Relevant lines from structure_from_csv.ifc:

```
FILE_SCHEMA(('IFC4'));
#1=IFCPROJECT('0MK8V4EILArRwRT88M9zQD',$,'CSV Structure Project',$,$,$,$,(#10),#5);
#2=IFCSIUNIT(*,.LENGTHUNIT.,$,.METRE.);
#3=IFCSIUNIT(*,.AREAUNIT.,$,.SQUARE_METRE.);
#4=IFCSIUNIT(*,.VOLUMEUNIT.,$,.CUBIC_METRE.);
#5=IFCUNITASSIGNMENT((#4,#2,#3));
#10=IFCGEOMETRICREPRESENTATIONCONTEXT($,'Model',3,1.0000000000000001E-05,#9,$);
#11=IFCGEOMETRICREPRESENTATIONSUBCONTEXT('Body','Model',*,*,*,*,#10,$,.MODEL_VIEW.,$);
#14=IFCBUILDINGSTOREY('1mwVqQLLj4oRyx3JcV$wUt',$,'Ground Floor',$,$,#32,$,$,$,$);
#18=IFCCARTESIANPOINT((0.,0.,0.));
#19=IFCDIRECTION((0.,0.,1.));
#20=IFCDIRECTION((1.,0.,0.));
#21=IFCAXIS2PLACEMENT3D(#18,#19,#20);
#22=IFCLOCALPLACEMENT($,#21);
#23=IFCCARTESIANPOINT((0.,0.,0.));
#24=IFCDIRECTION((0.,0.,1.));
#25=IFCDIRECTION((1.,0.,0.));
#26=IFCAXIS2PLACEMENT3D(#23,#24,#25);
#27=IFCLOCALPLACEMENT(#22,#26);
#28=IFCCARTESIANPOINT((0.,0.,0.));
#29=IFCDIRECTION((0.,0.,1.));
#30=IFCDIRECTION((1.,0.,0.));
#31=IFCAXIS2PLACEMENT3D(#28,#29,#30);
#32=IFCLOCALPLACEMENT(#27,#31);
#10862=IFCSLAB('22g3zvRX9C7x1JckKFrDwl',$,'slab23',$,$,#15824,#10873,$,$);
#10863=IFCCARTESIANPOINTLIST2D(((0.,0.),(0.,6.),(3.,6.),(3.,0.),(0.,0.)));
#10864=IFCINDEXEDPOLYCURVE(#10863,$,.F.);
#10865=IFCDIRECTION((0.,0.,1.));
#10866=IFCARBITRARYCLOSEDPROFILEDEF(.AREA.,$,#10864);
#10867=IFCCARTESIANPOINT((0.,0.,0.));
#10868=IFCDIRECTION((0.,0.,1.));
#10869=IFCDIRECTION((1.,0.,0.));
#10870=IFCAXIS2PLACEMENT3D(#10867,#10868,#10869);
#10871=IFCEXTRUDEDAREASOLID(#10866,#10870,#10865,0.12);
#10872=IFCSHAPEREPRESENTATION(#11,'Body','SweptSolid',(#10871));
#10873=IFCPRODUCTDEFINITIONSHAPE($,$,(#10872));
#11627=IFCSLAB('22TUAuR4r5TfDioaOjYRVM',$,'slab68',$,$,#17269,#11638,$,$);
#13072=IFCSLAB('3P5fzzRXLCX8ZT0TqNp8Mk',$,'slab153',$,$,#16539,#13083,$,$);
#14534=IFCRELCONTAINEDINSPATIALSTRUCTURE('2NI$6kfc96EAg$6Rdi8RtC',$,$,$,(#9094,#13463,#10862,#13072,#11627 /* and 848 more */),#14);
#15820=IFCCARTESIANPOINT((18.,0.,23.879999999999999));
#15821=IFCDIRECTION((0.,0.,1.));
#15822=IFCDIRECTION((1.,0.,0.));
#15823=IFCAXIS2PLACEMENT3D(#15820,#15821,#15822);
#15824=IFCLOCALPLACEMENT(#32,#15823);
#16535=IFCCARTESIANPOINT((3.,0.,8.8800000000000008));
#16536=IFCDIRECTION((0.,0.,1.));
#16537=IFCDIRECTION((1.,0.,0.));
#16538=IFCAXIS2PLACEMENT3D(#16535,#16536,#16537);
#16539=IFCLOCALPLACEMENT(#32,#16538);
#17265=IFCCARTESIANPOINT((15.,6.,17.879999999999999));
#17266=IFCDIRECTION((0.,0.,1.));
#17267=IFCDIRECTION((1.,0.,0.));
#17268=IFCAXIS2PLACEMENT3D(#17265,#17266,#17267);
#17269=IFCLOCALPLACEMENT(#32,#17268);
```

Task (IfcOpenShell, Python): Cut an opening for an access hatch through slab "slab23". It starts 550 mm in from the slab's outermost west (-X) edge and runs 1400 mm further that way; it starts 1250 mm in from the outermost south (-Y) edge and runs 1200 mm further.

```python
import numpy as np
import ifcopenshell
import ifcopenshell.api.feature
import ifcopenshell.api.geometry
import ifcopenshell.api.root
import ifcopenshell.geom
import ifcopenshell.util.placement
import ifcopenshell.util.representation
import ifcopenshell.util.shape
import ifcopenshell.util.unit

model = ifcopenshell.open("structure_from_csv.ifc")
unit_scale = ifcopenshell.util.unit.calculate_unit_scale(model)
settings = ifcopenshell.geom.settings()


def volume(element):
    """Net volume in cubic metres, openings subtracted."""
    shape = ifcopenshell.geom.create_shape(settings, element)
    return ifcopenshell.util.shape.get_volume(shape.geometry)


slab = model.by_guid("22g3zvRX9C7x1JckKFrDwl")
before = volume(slab)

# Extent in the slab's own axes, in metres. The edges named are its -X and -Y sides.
slab_shape = ifcopenshell.geom.create_shape(settings, slab)
vertices = ifcopenshell.util.shape.get_vertices(slab_shape.geometry)
x_min, y_min, bottom = vertices.min(axis=0)
top = vertices[:, 2].max()

opening = ifcopenshell.api.root.create_entity(model, ifc_class="IfcOpeningElement", name="Access hatch opening", predefined_type="OPENING")
context = ifcopenshell.util.representation.get_context(model, "Model", "Body", "MODEL_VIEW")
width, depth = 1.4, 1.2
outline = [(0.0, 0.0), (width, 0.0), (width, depth), (0.0, depth), (0.0, 0.0)]
# Overshoot both faces by 50 mm so the cut is clean.
shape = ifcopenshell.api.geometry.add_slab_representation(
    model, context=context, depth=top - bottom + 0.1, polyline=outline
)
ifcopenshell.api.geometry.assign_representation(model, product=opening, representation=shape)

matrix = ifcopenshell.util.placement.get_local_placement(slab.ObjectPlacement)
matrix[:, 3] = matrix @ np.append(np.array([x_min + 0.55, y_min + 1.25, bottom - 0.05]) / unit_scale, 1.0)
ifcopenshell.api.geometry.edit_object_placement(model, product=opening, matrix=matrix, is_si=False)
ifcopenshell.api.feature.add_feature(model, feature=opening, element=slab)

after = volume(slab)

print(f"slab volume {before:.3f} -> {after:.3f} m3")

model.write("structure_from_csv_edited.ifc")
```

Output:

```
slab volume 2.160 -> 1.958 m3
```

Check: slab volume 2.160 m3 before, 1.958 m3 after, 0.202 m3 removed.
